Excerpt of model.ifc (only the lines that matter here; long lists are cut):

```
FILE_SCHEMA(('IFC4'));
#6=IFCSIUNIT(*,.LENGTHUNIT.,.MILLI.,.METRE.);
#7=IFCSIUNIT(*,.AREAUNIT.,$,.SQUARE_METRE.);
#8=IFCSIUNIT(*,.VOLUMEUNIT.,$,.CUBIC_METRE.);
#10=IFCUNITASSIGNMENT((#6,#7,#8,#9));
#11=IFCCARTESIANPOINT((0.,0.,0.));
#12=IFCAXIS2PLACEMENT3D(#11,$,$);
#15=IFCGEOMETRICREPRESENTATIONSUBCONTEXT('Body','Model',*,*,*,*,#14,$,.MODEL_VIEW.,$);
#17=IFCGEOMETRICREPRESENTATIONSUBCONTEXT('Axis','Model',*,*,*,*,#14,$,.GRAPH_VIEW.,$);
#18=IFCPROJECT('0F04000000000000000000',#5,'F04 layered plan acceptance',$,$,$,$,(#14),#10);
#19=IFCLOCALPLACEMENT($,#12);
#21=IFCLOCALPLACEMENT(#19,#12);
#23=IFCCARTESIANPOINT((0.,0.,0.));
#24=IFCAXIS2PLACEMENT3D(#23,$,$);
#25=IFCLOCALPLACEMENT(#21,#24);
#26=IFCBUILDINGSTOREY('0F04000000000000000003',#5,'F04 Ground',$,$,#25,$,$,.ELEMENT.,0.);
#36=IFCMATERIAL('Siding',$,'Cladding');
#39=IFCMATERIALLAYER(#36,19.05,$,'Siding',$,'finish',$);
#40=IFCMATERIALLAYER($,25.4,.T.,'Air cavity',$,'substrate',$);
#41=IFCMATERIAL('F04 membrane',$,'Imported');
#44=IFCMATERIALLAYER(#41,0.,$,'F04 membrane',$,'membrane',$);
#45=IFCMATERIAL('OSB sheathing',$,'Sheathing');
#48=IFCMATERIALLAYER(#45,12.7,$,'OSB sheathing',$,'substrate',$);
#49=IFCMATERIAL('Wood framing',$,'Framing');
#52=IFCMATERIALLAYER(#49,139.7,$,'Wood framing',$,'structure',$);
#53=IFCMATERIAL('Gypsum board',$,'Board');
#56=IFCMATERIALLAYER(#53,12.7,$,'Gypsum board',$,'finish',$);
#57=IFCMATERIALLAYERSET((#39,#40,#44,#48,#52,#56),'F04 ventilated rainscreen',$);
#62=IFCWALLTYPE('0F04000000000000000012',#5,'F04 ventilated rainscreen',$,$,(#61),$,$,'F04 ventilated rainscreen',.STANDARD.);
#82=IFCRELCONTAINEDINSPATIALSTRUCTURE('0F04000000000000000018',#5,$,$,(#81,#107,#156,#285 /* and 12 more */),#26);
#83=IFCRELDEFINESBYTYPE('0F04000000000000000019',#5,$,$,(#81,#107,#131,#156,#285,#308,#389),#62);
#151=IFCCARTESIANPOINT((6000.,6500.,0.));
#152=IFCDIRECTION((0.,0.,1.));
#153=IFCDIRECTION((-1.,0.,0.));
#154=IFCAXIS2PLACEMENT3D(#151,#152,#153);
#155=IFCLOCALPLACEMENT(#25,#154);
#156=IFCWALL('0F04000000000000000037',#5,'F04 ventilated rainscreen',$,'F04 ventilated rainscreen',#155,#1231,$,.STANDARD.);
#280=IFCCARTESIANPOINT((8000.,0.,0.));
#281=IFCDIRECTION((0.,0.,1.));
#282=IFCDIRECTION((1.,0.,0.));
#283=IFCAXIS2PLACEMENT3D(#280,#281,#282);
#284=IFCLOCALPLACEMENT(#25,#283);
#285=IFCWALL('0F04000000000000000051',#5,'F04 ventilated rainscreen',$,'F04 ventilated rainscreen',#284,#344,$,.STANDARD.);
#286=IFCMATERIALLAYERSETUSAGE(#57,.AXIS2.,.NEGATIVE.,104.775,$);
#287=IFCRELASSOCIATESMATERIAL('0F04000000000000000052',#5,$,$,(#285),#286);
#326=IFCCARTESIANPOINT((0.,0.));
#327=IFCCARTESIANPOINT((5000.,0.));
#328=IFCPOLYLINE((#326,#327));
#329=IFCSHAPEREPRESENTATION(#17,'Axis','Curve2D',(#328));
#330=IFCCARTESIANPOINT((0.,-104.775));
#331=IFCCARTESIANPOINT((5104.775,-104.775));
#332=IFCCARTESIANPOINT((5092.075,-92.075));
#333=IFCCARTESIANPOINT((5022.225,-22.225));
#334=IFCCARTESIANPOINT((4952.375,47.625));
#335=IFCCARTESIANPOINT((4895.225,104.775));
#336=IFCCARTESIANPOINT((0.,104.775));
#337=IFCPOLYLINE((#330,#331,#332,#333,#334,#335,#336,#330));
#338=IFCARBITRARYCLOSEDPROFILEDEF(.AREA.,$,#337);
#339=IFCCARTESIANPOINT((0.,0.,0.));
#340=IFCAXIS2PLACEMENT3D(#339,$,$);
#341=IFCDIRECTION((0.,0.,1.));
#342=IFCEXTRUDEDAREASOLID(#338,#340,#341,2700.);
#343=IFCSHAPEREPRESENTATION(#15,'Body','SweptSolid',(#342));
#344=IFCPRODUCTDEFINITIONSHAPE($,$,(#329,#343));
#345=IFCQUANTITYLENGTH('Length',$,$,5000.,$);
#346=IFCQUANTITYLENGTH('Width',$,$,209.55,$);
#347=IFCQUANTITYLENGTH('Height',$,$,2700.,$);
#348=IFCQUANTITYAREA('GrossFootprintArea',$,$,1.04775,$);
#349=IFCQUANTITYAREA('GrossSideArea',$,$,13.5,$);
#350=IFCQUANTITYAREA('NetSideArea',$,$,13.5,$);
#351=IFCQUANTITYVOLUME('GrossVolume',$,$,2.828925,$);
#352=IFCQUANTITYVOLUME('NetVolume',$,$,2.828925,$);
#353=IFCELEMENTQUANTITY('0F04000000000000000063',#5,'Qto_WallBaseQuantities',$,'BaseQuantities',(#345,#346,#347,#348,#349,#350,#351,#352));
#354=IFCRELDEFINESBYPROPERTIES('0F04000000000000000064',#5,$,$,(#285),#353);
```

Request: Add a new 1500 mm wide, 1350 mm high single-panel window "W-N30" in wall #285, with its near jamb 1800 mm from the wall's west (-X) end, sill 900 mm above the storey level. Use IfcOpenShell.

```python
import numpy as np
import ifcopenshell
import ifcopenshell.api.feature
import ifcopenshell.api.geometry
import ifcopenshell.api.pset
import ifcopenshell.api.root
import ifcopenshell.api.spatial
import ifcopenshell.geom
import ifcopenshell.util.element
import ifcopenshell.util.placement
import ifcopenshell.util.representation
import ifcopenshell.util.shape
import ifcopenshell.util.unit

model = ifcopenshell.open("model.ifc")
unit_scale = ifcopenshell.util.unit.calculate_unit_scale(model)
area_scale = ifcopenshell.util.unit.calculate_unit_scale(model, "AREAUNIT")
volume_scale = ifcopenshell.util.unit.calculate_unit_scale(model, "VOLUMEUNIT")
settings = ifcopenshell.geom.settings()


def volume(element):
    """Net volume in cubic metres, openings subtracted."""
    shape = ifcopenshell.geom.create_shape(settings, element)
    return ifcopenshell.util.shape.get_volume(shape.geometry)


wall = model.by_guid("0F04000000000000000051")
storey = ifcopenshell.util.element.get_container(wall, ifc_class="IfcBuildingStorey")
context = ifcopenshell.util.representation.get_context(model, "Model", "Body", "MODEL_VIEW")
before = volume(wall)

width, height, from_end, sill = 1.5, 1.35, 1.8, 0.9  # metres

# The wall runs along its own X axis, and the end named is its -X end.
wall_shape = ifcopenshell.geom.create_shape(settings, wall)
x, y, z = ifcopenshell.util.shape.get_vertices(wall_shape.geometry).T
start = x.min() + from_end
face, thickness = float(y.min()), float(y.max() - y.min())
wall_matrix = ifcopenshell.util.placement.get_local_placement(wall.ObjectPlacement)
level = ifcopenshell.util.placement.get_local_placement(storey.ObjectPlacement)[2, 3]


def in_wall(x, y):
    """Placement at x, y metres in the wall's axes, at sill height."""
    matrix = wall_matrix.copy()
    matrix[:, 3] = wall_matrix @ np.array([x / unit_scale, y / unit_scale, 0.0, 1.0])
    matrix[2, 3] = level + sill / unit_scale
    return matrix


# Opening: a box that overshoots both wall faces by 50 mm.
opening = ifcopenshell.api.root.create_entity(model, ifc_class="IfcOpeningElement", predefined_type="OPENING")
box = ifcopenshell.api.geometry.add_wall_representation(
    model, context=context, length=width, height=height, thickness=thickness + 0.1
)
ifcopenshell.api.geometry.assign_representation(model, product=opening, representation=box)
ifcopenshell.api.geometry.edit_object_placement(model, product=opening, matrix=in_wall(start, face - 0.05), is_si=False)
ifcopenshell.api.feature.add_feature(model, feature=opening, element=wall)

window = ifcopenshell.api.root.create_entity(model, ifc_class="IfcWindow", name="W-N30", predefined_type="WINDOW")
window.OverallWidth, window.OverallHeight = width / unit_scale, height / unit_scale
window.PartitioningType = "SINGLE_PANEL"
body = ifcopenshell.api.geometry.add_window_representation(
    model,
    context=context,
    overall_width=window.OverallWidth,
    overall_height=window.OverallHeight,
    partition_type="SINGLE_PANEL",
)
ifcopenshell.api.geometry.assign_representation(model, product=window, representation=body)
ifcopenshell.api.spatial.assign_container(model, products=[window], relating_structure=storey)
ifcopenshell.api.feature.add_filling(model, opening=opening, element=window)

# Centre the window in the wall's thickness.
ifcopenshell.api.geometry.edit_object_placement(model, product=window, matrix=in_wall(start, face), is_si=False)
window_shape = ifcopenshell.geom.create_shape(settings, window)
depth = ifcopenshell.util.shape.get_vertices(window_shape.geometry)[:, 1]
offset = face + thickness / 2 - (depth.min() + depth.max()) / 2
ifcopenshell.api.geometry.edit_object_placement(model, product=window, matrix=in_wall(start, offset), is_si=False)

after = volume(wall)

# Update the wall's stored quantities.
qto = model.by_id(ifcopenshell.util.element.get_pset(wall, "Qto_WallBaseQuantities", should_inherit=False)["id"])
ifcopenshell.api.pset.edit_qto(model, qto=qto, properties={
    "NetSideArea": after / thickness / area_scale,
    "NetVolume": after / volume_scale,
})

print(f"wall volume {before:.3f} -> {after:.3f} m3")

model.write("model_rev.ifc")
```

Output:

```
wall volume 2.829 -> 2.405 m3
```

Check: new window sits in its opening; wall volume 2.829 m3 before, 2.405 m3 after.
